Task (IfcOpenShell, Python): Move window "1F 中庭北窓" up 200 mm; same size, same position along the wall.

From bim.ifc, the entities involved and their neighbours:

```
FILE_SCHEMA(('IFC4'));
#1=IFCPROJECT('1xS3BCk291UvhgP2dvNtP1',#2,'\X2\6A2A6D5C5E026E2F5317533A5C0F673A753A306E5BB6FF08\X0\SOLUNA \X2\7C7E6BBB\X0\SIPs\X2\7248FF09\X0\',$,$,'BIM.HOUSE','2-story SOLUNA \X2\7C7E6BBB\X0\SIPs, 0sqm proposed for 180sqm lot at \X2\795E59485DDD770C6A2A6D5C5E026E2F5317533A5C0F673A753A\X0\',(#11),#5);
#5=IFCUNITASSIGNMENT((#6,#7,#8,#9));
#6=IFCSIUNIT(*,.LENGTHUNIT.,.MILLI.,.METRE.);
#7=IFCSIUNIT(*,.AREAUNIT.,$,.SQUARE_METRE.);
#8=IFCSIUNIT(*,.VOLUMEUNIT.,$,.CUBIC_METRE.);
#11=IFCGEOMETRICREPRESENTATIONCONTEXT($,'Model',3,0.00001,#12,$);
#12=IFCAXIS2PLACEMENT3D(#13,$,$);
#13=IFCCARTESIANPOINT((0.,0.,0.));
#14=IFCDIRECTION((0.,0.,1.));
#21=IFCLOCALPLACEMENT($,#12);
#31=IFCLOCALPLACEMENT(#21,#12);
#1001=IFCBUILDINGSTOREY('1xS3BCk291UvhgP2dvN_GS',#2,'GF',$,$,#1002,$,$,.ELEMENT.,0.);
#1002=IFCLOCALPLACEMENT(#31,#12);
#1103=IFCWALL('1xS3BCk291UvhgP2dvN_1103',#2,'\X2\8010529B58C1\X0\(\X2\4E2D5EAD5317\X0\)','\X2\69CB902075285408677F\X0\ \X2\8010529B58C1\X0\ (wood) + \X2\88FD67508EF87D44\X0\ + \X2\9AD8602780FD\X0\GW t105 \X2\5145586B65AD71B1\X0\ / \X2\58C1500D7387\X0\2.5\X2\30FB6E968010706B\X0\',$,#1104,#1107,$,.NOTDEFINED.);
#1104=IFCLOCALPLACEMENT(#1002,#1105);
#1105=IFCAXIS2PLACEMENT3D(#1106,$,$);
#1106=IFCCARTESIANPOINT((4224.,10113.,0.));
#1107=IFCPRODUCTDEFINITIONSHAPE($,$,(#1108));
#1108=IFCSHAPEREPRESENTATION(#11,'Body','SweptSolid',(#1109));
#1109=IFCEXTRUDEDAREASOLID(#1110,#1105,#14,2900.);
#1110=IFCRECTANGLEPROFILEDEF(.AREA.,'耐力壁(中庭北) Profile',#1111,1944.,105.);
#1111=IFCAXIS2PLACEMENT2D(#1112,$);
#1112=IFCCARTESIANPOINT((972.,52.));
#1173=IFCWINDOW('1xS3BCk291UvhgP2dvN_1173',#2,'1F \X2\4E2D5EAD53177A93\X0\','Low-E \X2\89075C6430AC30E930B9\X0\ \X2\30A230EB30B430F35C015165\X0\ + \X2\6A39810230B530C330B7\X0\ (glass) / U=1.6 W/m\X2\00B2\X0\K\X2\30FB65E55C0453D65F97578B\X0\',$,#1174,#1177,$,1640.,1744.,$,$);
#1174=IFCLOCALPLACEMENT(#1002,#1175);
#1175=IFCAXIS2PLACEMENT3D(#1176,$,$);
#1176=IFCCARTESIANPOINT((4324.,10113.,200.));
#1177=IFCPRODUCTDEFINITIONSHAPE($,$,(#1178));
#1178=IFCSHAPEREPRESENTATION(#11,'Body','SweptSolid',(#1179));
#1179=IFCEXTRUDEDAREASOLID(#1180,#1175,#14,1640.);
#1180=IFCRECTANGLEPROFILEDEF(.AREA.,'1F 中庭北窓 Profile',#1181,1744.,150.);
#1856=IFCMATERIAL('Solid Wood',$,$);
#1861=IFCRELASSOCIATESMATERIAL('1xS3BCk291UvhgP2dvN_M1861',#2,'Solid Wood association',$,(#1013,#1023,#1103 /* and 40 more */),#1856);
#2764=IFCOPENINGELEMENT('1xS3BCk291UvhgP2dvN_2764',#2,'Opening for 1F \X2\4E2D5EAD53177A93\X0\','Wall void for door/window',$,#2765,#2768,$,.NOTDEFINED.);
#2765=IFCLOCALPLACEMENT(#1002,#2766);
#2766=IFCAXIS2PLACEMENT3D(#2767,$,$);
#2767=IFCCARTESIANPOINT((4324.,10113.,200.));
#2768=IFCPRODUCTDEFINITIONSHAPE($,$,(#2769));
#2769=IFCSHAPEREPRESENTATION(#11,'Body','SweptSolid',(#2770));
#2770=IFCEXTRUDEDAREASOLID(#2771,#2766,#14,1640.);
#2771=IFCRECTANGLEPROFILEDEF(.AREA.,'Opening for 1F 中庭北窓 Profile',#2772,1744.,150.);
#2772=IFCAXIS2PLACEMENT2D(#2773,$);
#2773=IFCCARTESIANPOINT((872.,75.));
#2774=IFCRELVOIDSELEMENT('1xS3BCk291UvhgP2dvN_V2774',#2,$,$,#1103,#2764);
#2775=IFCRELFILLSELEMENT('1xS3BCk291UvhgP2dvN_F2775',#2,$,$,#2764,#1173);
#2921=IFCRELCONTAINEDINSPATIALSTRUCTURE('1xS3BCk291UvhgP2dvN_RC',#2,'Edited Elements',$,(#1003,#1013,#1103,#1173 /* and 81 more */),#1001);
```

```python
import numpy as np
import ifcopenshell
import ifcopenshell.api.geometry
import ifcopenshell.util.placement
import ifcopenshell.util.unit

model = ifcopenshell.open("bim.ifc")
unit_scale = ifcopenshell.util.unit.calculate_unit_scale(model)

window = model.by_guid("1xS3BCk291UvhgP2dvN_1173")
opening = window.FillsVoids[0].RelatingOpeningElement
dz = 0.2 / unit_scale

shift = np.array([0.0, 0.0, dz])
# The window is not placed relative to its opening, so move both.
for product in (opening, window):
    matrix = ifcopenshell.util.placement.get_local_placement(product.ObjectPlacement)
    matrix[:3, 3] += shift
    ifcopenshell.api.geometry.edit_object_placement(model, product=product, matrix=matrix, is_si=False)

print(f"moved by {dz * unit_scale:+.3f} m")

model.write("bim_v2.ifc")
```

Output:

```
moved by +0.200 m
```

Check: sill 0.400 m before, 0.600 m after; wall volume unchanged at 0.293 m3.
